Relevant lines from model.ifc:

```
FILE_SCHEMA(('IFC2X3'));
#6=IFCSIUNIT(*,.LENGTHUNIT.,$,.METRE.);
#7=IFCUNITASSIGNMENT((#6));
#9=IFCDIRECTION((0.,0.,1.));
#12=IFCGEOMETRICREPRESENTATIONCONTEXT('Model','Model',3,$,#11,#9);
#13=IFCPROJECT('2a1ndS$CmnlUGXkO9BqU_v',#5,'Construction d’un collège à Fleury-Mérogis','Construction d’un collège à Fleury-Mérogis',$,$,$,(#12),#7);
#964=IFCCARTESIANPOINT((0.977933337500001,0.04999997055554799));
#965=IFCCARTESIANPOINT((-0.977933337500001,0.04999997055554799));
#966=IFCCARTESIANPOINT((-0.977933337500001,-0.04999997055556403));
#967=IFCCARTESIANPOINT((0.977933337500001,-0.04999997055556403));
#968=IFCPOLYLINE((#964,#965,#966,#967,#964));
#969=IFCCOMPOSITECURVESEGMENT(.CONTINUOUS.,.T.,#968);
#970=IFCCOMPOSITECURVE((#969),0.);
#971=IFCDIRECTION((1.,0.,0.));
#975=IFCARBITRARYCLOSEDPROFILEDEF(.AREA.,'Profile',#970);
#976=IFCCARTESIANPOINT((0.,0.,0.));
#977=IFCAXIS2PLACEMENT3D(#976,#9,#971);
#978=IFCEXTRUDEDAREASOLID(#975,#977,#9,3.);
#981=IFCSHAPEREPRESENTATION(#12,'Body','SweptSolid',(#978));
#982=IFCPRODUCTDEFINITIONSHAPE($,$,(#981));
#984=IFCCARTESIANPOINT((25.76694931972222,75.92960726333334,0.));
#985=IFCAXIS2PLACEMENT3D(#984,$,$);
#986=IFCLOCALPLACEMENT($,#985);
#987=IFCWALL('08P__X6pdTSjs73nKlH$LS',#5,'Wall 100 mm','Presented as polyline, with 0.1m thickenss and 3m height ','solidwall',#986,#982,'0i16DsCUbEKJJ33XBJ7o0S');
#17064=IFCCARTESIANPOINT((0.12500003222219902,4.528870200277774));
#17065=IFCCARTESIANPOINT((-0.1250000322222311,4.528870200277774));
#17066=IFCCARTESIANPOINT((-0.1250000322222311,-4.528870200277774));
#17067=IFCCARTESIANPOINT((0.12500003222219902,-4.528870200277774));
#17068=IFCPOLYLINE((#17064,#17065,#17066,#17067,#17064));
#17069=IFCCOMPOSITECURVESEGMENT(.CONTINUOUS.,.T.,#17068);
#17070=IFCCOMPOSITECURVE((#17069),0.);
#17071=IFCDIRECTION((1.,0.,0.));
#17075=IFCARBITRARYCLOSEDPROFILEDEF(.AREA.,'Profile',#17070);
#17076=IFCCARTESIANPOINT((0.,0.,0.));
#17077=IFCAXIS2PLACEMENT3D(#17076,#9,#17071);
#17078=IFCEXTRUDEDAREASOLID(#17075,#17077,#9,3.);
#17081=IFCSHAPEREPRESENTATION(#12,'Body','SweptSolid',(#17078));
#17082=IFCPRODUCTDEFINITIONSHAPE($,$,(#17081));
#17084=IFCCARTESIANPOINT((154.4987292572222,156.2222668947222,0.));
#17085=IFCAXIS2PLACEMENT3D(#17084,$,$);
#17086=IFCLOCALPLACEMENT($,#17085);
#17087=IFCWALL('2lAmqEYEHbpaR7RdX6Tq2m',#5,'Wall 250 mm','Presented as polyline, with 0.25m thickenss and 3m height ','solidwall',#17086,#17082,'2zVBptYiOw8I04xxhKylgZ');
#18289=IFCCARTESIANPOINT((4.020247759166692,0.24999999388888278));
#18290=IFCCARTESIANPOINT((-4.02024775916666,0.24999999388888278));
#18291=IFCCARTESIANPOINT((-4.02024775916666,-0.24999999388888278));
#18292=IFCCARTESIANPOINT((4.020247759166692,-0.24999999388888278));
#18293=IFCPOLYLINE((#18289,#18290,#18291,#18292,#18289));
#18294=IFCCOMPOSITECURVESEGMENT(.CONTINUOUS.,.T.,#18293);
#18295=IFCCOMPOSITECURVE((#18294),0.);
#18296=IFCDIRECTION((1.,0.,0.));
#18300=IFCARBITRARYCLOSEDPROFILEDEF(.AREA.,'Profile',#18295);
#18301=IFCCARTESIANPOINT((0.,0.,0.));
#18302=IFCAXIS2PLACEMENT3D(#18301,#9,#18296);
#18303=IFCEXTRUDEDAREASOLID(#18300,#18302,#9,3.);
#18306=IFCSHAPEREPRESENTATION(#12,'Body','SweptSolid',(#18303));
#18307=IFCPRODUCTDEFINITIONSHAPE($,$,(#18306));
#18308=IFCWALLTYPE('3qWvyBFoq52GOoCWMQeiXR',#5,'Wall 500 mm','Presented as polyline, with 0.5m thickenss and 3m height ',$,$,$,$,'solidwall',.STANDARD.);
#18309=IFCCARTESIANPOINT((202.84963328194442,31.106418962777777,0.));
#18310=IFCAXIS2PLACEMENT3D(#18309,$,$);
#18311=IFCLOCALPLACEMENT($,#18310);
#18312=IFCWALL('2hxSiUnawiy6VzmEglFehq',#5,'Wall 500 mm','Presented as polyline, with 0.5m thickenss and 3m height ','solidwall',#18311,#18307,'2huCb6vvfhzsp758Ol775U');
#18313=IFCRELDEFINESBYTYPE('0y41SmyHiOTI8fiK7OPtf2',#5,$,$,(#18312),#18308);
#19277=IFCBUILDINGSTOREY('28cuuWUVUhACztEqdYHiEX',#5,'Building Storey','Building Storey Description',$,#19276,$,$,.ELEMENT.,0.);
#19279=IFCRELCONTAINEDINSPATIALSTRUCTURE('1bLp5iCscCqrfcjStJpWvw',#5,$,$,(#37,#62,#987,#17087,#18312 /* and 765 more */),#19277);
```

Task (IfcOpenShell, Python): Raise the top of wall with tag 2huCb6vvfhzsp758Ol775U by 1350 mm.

```python
import ifcopenshell
import ifcopenshell.geom
import ifcopenshell.util.shape

model = ifcopenshell.open("model.ifc")
settings = ifcopenshell.geom.settings()


def volume(element):
    """Net volume in cubic metres, openings subtracted."""
    shape = ifcopenshell.geom.create_shape(settings, element)
    return ifcopenshell.util.shape.get_volume(shape.geometry)


wall = model.by_guid("2hxSiUnawiy6VzmEglFehq")
before = volume(wall)

body = next(r for r in wall.Representation.Representations if r.RepresentationIdentifier == "Body")
solid = body.Items[0]
old_height = solid.Depth
solid.Depth += 1.35
after = volume(wall)

print(f"height {old_height:g} -> {solid.Depth:g}, volume {before:.3f} -> {after:.3f} m3")

model.write("model_updated.ifc")
```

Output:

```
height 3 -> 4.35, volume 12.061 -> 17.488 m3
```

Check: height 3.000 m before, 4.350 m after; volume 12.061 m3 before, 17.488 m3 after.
